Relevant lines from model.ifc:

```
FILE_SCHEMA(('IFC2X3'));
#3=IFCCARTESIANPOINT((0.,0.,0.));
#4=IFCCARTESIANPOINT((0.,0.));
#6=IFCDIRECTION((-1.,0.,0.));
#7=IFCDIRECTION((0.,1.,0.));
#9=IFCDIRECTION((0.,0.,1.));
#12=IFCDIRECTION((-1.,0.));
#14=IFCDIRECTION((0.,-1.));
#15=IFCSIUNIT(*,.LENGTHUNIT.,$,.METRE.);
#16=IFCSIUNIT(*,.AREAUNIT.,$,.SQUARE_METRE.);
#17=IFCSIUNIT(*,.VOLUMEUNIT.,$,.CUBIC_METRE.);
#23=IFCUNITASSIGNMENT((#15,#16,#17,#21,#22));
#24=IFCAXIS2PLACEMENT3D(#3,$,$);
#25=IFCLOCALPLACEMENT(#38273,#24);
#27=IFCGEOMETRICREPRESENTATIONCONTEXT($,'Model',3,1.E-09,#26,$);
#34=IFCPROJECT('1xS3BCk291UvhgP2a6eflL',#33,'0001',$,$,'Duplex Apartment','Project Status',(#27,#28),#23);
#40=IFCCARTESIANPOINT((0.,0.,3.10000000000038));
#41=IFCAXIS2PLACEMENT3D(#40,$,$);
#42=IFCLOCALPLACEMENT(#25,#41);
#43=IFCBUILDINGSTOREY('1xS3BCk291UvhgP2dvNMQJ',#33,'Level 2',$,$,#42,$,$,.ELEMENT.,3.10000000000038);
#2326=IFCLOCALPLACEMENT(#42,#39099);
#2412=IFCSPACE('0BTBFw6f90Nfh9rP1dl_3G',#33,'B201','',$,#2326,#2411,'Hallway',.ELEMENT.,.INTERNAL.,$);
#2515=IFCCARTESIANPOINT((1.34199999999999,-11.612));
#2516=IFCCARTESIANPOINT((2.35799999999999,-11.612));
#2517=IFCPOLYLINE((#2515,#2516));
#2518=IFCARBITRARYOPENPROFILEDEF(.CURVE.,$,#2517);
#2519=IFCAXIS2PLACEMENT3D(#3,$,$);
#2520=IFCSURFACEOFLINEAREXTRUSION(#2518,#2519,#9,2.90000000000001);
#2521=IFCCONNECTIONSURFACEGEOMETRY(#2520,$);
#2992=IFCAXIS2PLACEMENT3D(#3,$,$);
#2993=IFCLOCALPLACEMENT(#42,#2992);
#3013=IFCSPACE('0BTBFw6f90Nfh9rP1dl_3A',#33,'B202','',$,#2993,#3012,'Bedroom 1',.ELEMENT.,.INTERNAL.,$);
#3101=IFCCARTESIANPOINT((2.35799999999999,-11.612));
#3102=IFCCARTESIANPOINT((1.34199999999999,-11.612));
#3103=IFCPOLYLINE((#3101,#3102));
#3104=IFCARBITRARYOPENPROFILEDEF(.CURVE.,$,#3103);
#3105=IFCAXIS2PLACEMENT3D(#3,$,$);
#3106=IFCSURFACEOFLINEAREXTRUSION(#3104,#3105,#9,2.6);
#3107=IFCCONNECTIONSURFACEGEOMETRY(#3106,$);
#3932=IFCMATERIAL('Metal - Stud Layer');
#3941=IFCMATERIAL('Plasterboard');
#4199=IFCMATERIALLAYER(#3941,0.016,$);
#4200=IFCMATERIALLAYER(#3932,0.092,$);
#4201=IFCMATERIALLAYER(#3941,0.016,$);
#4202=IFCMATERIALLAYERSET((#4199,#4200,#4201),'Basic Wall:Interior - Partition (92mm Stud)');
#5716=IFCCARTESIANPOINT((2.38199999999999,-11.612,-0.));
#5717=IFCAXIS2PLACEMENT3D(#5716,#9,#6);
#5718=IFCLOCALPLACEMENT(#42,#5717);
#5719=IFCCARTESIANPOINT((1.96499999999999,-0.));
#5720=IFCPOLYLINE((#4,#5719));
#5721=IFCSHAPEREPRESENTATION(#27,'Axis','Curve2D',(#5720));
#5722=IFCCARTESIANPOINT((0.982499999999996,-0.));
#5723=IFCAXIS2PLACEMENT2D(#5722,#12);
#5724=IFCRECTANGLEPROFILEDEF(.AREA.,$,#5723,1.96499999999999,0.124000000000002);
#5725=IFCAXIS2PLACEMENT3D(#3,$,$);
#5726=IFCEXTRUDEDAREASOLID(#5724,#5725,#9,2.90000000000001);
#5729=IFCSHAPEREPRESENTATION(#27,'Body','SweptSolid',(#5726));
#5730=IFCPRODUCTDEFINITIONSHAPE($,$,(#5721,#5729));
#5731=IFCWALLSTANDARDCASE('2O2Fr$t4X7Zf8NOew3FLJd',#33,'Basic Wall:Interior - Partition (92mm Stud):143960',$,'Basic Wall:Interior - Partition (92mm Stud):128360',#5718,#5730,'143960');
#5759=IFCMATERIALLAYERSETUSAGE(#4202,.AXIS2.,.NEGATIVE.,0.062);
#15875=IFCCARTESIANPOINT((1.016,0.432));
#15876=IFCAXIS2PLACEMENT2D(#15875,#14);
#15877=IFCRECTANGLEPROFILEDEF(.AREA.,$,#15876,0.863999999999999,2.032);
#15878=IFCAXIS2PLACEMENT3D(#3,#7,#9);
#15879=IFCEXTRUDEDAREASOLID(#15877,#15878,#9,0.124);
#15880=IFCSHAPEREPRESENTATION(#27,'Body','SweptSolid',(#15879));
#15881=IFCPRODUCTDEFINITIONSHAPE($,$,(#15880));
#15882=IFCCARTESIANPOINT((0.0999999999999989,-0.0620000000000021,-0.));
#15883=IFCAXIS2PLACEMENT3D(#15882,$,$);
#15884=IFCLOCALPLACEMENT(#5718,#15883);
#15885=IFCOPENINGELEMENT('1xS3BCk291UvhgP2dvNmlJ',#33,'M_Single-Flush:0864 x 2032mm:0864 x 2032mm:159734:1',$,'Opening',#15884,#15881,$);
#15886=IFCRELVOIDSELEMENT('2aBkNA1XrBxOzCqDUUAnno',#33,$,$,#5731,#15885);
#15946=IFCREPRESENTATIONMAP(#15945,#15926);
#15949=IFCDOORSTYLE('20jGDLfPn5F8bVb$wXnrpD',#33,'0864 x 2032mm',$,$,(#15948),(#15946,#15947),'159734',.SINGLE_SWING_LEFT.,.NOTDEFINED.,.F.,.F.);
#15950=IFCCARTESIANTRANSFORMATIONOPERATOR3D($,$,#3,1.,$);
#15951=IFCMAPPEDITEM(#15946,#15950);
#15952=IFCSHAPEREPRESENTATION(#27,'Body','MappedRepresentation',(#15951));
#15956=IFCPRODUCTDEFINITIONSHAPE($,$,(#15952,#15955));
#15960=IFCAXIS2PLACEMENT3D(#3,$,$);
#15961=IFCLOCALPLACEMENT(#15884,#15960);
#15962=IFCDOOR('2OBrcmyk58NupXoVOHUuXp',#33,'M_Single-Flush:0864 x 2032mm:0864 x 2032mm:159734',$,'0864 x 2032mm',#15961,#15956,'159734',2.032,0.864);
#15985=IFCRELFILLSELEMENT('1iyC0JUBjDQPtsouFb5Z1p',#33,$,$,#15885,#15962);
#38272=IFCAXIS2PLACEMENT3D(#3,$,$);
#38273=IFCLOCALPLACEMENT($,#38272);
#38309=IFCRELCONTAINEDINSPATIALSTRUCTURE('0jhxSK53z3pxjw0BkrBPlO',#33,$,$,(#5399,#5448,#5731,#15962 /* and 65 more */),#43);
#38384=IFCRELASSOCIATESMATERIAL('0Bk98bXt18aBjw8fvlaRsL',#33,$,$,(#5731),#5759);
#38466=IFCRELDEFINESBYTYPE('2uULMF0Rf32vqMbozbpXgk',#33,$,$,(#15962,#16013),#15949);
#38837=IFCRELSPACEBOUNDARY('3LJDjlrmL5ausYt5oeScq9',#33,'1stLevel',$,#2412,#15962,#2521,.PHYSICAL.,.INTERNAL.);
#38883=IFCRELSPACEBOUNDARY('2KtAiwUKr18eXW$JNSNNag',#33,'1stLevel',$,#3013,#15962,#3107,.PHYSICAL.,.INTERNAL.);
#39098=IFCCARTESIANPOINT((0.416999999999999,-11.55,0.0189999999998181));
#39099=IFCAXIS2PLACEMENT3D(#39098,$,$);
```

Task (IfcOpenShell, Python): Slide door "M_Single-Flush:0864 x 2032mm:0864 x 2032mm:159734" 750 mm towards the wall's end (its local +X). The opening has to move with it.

```python
import numpy as np
import ifcopenshell
import ifcopenshell.api.geometry
import ifcopenshell.util.placement
import ifcopenshell.util.unit

model = ifcopenshell.open("model.ifc")
unit_scale = ifcopenshell.util.unit.calculate_unit_scale(model)

door = model.by_id(15962)
opening = door.FillsVoids[0].RelatingOpeningElement
wall = opening.VoidsElements[0].RelatingBuildingElement

wall_matrix = ifcopenshell.util.placement.get_local_placement(wall.ObjectPlacement)
shift = wall_matrix[:3, 0] * 0.75 / unit_scale
before = ifcopenshell.util.placement.get_local_placement(door.ObjectPlacement)[:3, 3].copy()

# The door is placed relative to its opening, so it follows when the opening moves.
matrix = ifcopenshell.util.placement.get_local_placement(opening.ObjectPlacement)
matrix[:3, 3] += shift
ifcopenshell.api.geometry.edit_object_placement(
    model, product=opening, matrix=matrix, is_si=False, should_transform_children=True
)

# Space boundary surfaces are stored in each space's coordinates; move them too.
for rel in door.ProvidesBoundaries:
    if not rel.ConnectionGeometry:
        continue
    surface = rel.ConnectionGeometry.SurfaceOnRelatingElement
    space_matrix = ifcopenshell.util.placement.get_local_placement(rel.RelatingSpace.ObjectPlacement)
    point = np.array(surface.Position.Location.Coordinates) + space_matrix[:3, :3].T @ shift
    surface.Position = model.createIfcAxis2Placement3D(
        model.createIfcCartesianPoint(point.tolist()), surface.Position.Axis, surface.Position.RefDirection
    )

after = ifcopenshell.util.placement.get_local_placement(door.ObjectPlacement)[:3, 3]
print("door moved by", (after - before).round(3) + 0.0)

model.write("model_v2.ifc")
```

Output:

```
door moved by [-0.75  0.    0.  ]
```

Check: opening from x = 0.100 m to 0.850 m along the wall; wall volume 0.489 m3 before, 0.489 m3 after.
